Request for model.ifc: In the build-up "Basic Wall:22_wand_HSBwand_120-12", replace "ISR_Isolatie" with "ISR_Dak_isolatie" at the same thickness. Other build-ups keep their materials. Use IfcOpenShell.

First a look at what the model holds.

```python
import ifcopenshell
import ifcopenshell.util.element

model = ifcopenshell.open("model.ifc")
print(model.schema)
for layer_set in model.by_type("IfcMaterialLayerSet"):
    if layer_set.LayerSetName == "Basic Wall:22_wand_HSBwand_120-12":
        for layer in layer_set.MaterialLayers:
            print(layer.id(), layer.Material and layer.Material.Name, layer.LayerThickness, sep=" | ")
        print(len(ifcopenshell.util.element.get_elements_by_material(model, layer_set)), "elements and types use it")
print(sorted(m.Name for m in model.by_type("IfcMaterial") if m.Name)[:60])
```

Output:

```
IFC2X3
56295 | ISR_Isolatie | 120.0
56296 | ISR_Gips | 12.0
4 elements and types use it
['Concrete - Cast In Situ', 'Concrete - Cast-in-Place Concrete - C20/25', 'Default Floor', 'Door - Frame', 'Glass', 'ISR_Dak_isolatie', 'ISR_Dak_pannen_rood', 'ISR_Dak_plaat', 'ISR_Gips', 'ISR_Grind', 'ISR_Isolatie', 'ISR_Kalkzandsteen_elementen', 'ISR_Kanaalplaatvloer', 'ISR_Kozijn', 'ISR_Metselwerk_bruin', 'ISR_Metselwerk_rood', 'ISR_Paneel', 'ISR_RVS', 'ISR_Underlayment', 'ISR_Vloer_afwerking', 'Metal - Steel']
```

```python
import ifcopenshell
import ifcopenshell.api.material

model = ifcopenshell.open("model.ifc")

layer_set = next(s for s in model.by_type("IfcMaterialLayerSet") if s.LayerSetName == "Basic Wall:22_wand_HSBwand_120-12")
layer = next(l for l in layer_set.MaterialLayers if l.Material and l.Material.Name == "ISR_Isolatie")
material = next(m for m in model.by_type("IfcMaterial") if m.Name == "ISR_Dak_isolatie")

# Point this one layer at the other material; renaming the old one would change it everywhere.
ifcopenshell.api.material.edit_layer(model, layer=layer, attributes={}, material=material)

print([l.Material.Name if l.Material else None for l in layer_set.MaterialLayers])

model.write("model_v2.ifc")
```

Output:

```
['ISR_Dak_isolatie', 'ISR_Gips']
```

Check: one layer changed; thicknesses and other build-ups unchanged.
